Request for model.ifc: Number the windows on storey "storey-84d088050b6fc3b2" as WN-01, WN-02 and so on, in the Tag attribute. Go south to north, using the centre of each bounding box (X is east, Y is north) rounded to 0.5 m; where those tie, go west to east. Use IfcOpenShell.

First a look at what the model holds.

```python
import ifcopenshell
import ifcopenshell.util.element
import ifcopenshell.util.placement

model = ifcopenshell.open("model.ifc")
print(model.schema)
storey = next(s for s in model.by_type("IfcBuildingStorey") if s.Name == "storey-84d088050b6fc3b2")
windows = [e for e in ifcopenshell.util.element.get_decomposition(storey) if e.is_a("IfcWindow")]
for e in sorted(windows, key=lambda e: e.id()):
    origin = ifcopenshell.util.placement.get_local_placement(e.ObjectPlacement)[:3, 3]
    print(e.id(), e.Tag, e.Name, origin.round(2) + 0.0, sep=" | ")
```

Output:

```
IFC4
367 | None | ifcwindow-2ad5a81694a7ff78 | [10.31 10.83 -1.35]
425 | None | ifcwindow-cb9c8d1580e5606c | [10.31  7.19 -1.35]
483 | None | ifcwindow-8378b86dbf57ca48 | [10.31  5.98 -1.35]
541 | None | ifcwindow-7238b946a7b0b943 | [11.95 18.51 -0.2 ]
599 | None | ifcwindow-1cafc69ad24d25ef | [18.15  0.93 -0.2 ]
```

```python
import ifcopenshell
import ifcopenshell.geom
import ifcopenshell.util.element
import ifcopenshell.util.shape

model = ifcopenshell.open("model.ifc")
settings = ifcopenshell.geom.settings()
settings.set("use-world-coords", True)


def centre(element):
    shape = ifcopenshell.geom.create_shape(settings, element)
    return ifcopenshell.util.shape.get_bbox_centroid(shape.geometry)


storey = next(s for s in model.by_type("IfcBuildingStorey") if s.Name == "storey-84d088050b6fc3b2")
windows = [e for e in ifcopenshell.util.element.get_decomposition(storey) if e.is_a("IfcWindow")]

# Insertion points can sit at a corner or the storey origin, so sort by the geometry (in metres).
centres = {e: centre(e) for e in windows}
windows.sort(key=lambda e: (round(centres[e][1] / 0.5), centres[e][0]))

for i, e in enumerate(windows, start=1):
    number = f"WN-{i:02d}"
    e.Tag = number
    print(e.id(), number)

model.write("model_v2.ifc")
```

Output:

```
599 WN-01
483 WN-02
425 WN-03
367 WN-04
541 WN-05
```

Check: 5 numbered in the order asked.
